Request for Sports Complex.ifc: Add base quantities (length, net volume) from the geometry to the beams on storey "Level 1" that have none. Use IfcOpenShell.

First a look at what the model holds.

```python
import ifcopenshell
import ifcopenshell.util.element
import ifcopenshell.util.unit

model = ifcopenshell.open("Sports Complex.ifc")
print(model.schema)
for unit_type in ("LENGTHUNIT", "AREAUNIT", "VOLUMEUNIT"):
    print(unit_type, ifcopenshell.util.unit.calculate_unit_scale(model, unit_type))
storey = next(s for s in model.by_type("IfcBuildingStorey") if s.Name == "Level 1")
beams = [e for e in ifcopenshell.util.element.get_decomposition(storey) if e.is_a("IfcBeam")]
for e in sorted(beams, key=lambda e: e.id()):
    print(e.id(), e.is_a(), e.Name, list(ifcopenshell.util.element.get_psets(e, qtos_only=True)), sep=" | ")
```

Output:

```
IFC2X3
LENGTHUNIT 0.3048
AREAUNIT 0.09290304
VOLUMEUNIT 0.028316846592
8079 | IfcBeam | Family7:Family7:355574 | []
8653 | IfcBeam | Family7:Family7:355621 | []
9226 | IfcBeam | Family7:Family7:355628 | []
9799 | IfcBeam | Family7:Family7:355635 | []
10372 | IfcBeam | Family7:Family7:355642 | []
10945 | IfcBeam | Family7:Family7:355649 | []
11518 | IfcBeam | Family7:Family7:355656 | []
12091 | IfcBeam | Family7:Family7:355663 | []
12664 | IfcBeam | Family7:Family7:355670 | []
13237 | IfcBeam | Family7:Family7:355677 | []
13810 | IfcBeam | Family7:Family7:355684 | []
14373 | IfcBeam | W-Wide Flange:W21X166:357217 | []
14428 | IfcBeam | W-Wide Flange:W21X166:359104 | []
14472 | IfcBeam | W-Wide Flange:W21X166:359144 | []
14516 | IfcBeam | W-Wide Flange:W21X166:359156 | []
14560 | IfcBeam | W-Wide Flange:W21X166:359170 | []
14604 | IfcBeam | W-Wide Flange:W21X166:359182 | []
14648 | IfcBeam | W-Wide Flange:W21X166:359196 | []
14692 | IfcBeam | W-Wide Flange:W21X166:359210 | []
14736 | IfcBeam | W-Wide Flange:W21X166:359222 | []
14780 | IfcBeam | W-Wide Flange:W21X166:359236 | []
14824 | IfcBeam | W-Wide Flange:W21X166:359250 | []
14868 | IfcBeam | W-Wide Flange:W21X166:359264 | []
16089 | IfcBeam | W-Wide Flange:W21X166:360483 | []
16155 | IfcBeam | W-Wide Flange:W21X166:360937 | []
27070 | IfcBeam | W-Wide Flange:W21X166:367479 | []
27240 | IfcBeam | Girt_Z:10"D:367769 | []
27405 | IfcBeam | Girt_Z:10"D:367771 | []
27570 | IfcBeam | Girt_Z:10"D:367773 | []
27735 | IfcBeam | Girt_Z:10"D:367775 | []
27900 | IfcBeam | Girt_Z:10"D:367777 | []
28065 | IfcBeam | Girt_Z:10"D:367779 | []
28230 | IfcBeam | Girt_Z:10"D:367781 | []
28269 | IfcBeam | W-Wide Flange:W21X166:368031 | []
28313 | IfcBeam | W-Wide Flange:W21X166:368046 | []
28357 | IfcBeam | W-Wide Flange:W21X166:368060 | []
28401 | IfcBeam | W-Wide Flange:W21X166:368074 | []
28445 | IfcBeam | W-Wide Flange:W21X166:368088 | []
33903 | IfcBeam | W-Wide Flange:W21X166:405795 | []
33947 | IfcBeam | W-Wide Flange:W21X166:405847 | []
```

```python
import ifcopenshell
import ifcopenshell.api.pset
import ifcopenshell.geom
import ifcopenshell.util.element
import ifcopenshell.util.shape
import ifcopenshell.util.unit

model = ifcopenshell.open("Sports Complex.ifc")
unit_scale = ifcopenshell.util.unit.calculate_unit_scale(model)
volume_scale = ifcopenshell.util.unit.calculate_unit_scale(model, "VOLUMEUNIT")
settings = ifcopenshell.geom.settings()

storey = next(s for s in model.by_type("IfcBuildingStorey") if s.Name == "Level 1")
beams = [e for e in ifcopenshell.util.element.get_decomposition(storey) if e.is_a("IfcBeam")]

for e in sorted(beams, key=lambda e: e.id()):
    if ifcopenshell.util.element.get_psets(e, qtos_only=True, should_inherit=False):
        continue
    # Geometry comes back in metres, in the element's own axes.
    shape = ifcopenshell.geom.create_shape(settings, e)
    values = {
        "Length": ifcopenshell.util.shape.get_max_xyz(shape.geometry) / unit_scale,
        "NetVolume": ifcopenshell.util.shape.get_volume(shape.geometry) / volume_scale,
    }
    qto = ifcopenshell.api.pset.add_qto(model, product=e, name="BaseQuantities")
    ifcopenshell.api.pset.edit_qto(model, qto=qto, properties=values)
    print(e.id(), {k: round(v, 3) for k, v in values.items()})

model.write("Sports Complex-out.ifc")
```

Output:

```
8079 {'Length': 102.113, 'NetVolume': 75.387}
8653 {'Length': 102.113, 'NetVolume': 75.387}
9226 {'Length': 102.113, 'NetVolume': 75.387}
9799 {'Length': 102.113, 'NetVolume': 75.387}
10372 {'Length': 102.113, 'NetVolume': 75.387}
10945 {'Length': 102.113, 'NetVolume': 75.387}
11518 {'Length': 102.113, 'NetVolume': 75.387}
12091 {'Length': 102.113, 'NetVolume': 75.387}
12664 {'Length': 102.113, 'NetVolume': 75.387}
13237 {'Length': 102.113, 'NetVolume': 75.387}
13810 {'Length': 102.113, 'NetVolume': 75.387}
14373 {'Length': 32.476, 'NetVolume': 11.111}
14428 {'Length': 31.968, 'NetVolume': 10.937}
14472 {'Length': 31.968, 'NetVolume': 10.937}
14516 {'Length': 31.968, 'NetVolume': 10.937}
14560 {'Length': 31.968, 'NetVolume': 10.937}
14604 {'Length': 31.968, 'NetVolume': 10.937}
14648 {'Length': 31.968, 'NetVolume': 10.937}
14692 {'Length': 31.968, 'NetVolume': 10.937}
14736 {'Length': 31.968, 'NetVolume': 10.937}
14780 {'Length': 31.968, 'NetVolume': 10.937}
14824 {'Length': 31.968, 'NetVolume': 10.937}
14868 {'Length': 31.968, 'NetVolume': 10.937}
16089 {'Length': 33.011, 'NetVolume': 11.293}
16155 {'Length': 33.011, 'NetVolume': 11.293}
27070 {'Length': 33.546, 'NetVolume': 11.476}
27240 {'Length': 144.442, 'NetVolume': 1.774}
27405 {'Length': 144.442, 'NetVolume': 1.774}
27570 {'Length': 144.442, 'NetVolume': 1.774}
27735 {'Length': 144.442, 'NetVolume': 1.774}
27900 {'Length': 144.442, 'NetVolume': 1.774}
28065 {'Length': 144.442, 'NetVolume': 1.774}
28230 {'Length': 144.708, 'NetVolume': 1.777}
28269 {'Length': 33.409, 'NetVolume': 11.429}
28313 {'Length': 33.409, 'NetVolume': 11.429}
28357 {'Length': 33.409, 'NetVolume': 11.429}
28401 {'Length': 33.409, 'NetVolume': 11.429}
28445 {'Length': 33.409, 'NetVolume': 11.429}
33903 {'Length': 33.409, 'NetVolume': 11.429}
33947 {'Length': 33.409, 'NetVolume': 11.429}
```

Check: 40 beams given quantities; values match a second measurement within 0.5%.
